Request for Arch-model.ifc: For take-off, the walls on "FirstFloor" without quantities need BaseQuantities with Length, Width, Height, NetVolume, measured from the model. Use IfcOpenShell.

First a look at what the model holds.

```python
import ifcopenshell
import ifcopenshell.util.element
import ifcopenshell.util.unit

model = ifcopenshell.open("Arch-model.ifc")
print(model.schema)
for unit_type in ("LENGTHUNIT", "AREAUNIT", "VOLUMEUNIT"):
    print(unit_type, ifcopenshell.util.unit.calculate_unit_scale(model, unit_type))
storey = next(s for s in model.by_type("IfcBuildingStorey") if s.Name == "FirstFloor")
walls = [e for e in ifcopenshell.util.element.get_decomposition(storey) if e.is_a("IfcWall")]
for e in sorted(walls, key=lambda e: e.id()):
    print(e.id(), e.is_a(), e.Name, list(ifcopenshell.util.element.get_psets(e, qtos_only=True)), sep=" | ")
```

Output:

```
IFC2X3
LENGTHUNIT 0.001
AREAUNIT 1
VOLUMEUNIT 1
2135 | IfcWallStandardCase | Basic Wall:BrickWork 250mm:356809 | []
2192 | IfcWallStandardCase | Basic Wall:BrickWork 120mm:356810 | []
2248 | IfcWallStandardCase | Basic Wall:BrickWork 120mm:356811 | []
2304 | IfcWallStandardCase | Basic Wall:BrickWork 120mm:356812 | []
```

```python
import ifcopenshell
import ifcopenshell.api.pset
import ifcopenshell.geom
import ifcopenshell.util.element
import ifcopenshell.util.shape
import ifcopenshell.util.unit

model = ifcopenshell.open("Arch-model.ifc")
unit_scale = ifcopenshell.util.unit.calculate_unit_scale(model)
volume_scale = ifcopenshell.util.unit.calculate_unit_scale(model, "VOLUMEUNIT")
settings = ifcopenshell.geom.settings()

storey = next(s for s in model.by_type("IfcBuildingStorey") if s.Name == "FirstFloor")
walls = [e for e in ifcopenshell.util.element.get_decomposition(storey) if e.is_a("IfcWall")]

for e in sorted(walls, key=lambda e: e.id()):
    if ifcopenshell.util.element.get_psets(e, qtos_only=True, should_inherit=False):
        continue
    # Geometry comes back in metres, in the element's own axes.
    shape = ifcopenshell.geom.create_shape(settings, e)
    values = {
        "Length": ifcopenshell.util.shape.get_x(shape.geometry) / unit_scale,
        "Width": ifcopenshell.util.shape.get_y(shape.geometry) / unit_scale,
        "Height": ifcopenshell.util.shape.get_z(shape.geometry) / unit_scale,
        "NetVolume": ifcopenshell.util.shape.get_volume(shape.geometry) / volume_scale,
    }
    qto = ifcopenshell.api.pset.add_qto(model, product=e, name="BaseQuantities")
    ifcopenshell.api.pset.edit_qto(model, qto=qto, properties=values)
    print(e.id(), {k: round(v, 3) for k, v in values.items()})

model.write("Arch-model_edited.ifc")
```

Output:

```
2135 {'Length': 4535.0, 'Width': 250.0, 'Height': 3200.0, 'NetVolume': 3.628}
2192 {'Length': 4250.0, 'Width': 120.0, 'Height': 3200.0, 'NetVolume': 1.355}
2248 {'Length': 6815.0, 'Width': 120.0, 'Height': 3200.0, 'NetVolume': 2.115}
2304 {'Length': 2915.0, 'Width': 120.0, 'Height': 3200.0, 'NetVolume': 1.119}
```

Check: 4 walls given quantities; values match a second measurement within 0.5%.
